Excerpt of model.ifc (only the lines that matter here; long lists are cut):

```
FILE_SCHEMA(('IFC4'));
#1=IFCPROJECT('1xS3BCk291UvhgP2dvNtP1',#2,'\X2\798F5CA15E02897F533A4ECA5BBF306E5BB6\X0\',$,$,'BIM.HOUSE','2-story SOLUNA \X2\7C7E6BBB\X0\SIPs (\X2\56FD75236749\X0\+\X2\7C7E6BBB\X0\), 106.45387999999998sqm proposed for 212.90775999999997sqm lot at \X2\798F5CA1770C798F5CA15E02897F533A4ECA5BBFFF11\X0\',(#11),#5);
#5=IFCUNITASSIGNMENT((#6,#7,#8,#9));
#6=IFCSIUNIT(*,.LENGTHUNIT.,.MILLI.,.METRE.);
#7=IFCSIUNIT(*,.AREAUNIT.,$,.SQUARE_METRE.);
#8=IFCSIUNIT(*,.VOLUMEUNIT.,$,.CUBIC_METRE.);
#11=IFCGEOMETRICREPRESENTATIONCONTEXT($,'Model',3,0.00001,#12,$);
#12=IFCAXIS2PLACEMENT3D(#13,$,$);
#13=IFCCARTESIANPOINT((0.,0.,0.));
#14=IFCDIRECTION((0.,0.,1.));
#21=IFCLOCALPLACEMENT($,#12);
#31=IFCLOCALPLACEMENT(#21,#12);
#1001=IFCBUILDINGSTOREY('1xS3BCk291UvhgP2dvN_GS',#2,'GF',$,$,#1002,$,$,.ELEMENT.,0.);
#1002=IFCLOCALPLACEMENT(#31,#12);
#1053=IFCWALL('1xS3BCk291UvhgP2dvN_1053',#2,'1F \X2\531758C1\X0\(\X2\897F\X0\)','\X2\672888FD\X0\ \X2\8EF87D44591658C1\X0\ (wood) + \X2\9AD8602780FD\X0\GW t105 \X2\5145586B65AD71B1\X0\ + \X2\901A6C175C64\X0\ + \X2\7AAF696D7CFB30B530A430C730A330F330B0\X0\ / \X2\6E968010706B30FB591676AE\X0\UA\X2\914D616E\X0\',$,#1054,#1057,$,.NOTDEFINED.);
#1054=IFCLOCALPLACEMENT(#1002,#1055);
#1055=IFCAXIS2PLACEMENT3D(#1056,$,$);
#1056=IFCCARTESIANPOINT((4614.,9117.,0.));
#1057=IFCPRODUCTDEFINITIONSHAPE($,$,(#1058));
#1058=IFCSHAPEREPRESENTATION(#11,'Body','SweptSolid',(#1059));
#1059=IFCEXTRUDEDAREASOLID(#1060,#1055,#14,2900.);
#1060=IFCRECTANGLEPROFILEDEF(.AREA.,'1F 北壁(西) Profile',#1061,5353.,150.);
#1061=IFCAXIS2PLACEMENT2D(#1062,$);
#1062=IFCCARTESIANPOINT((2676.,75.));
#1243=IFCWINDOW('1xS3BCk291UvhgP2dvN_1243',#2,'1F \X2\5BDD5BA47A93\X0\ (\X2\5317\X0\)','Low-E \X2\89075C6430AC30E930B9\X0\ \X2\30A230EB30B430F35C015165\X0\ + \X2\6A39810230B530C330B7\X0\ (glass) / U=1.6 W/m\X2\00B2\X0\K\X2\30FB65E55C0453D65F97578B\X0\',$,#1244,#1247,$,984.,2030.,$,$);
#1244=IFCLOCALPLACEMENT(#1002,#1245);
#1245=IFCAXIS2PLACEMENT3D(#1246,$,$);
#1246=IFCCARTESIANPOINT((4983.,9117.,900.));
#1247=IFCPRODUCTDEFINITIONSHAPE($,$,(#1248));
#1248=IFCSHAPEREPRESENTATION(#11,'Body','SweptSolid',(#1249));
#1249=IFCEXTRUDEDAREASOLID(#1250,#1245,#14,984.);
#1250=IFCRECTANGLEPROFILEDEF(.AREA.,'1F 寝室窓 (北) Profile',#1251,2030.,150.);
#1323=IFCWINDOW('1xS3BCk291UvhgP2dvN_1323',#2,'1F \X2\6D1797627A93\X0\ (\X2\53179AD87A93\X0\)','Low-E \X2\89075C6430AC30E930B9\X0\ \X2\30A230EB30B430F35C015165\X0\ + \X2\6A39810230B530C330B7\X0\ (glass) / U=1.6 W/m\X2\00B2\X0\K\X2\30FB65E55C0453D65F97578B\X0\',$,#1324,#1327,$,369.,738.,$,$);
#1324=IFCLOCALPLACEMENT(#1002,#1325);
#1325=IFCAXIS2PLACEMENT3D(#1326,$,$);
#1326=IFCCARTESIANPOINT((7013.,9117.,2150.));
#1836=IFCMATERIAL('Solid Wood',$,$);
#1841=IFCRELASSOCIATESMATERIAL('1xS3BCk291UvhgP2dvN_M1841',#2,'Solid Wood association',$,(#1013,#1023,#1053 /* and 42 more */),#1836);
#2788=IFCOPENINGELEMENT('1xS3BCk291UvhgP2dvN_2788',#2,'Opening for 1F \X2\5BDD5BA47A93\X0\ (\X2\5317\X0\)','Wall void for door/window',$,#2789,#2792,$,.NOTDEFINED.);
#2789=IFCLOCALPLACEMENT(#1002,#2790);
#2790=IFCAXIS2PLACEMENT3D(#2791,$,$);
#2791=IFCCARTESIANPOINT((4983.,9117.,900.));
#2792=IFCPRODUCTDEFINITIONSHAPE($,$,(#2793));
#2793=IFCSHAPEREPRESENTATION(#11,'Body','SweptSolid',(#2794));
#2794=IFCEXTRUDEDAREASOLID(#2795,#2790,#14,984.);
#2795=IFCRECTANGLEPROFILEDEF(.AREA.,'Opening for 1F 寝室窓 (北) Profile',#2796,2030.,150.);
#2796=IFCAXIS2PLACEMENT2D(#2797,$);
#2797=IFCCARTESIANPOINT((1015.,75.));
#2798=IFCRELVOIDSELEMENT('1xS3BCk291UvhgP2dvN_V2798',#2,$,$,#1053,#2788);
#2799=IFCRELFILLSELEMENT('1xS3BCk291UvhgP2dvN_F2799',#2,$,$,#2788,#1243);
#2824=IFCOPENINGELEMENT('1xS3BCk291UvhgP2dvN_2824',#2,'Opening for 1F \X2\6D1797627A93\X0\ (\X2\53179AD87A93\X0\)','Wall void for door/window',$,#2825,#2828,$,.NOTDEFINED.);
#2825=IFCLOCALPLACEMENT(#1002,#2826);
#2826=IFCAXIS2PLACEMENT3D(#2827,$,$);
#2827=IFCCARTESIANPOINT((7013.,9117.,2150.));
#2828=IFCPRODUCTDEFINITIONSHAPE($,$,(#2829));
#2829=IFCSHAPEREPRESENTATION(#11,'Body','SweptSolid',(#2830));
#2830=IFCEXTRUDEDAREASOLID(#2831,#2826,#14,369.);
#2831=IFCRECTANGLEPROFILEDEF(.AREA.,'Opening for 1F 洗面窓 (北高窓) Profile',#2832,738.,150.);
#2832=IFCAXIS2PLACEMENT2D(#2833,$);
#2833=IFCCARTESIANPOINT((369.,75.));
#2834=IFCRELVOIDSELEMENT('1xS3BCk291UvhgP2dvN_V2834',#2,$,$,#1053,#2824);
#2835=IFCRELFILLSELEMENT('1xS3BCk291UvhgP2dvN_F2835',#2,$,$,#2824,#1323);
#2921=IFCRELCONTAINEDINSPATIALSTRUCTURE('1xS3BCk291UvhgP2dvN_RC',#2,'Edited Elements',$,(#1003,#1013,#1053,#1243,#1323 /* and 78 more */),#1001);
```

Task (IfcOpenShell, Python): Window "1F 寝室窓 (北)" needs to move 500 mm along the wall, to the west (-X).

```python
import ifcopenshell
import ifcopenshell.api.geometry
import ifcopenshell.util.placement

model = ifcopenshell.open("model.ifc")

window = model.by_guid("1xS3BCk291UvhgP2dvN_1243")
opening = window.FillsVoids[0].RelatingOpeningElement
wall = opening.VoidsElements[0].RelatingBuildingElement

wall_matrix = ifcopenshell.util.placement.get_local_placement(wall.ObjectPlacement)
shift = wall_matrix[:3, 0] * -500.0
before = ifcopenshell.util.placement.get_local_placement(window.ObjectPlacement)[:3, 3].copy()

# The window is not placed relative to its opening, so move both.
for product in (opening, window):
    matrix = ifcopenshell.util.placement.get_local_placement(product.ObjectPlacement)
    matrix[:3, 3] += shift
    ifcopenshell.api.geometry.edit_object_placement(model, product=product, matrix=matrix, is_si=False)

after = ifcopenshell.util.placement.get_local_placement(window.ObjectPlacement)[:3, 3]
print("window moved by", (after - before).round(3) + 0.0)

model.write("model_v2.ifc")
```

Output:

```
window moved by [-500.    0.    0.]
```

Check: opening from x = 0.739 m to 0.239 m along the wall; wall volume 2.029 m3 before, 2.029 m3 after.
